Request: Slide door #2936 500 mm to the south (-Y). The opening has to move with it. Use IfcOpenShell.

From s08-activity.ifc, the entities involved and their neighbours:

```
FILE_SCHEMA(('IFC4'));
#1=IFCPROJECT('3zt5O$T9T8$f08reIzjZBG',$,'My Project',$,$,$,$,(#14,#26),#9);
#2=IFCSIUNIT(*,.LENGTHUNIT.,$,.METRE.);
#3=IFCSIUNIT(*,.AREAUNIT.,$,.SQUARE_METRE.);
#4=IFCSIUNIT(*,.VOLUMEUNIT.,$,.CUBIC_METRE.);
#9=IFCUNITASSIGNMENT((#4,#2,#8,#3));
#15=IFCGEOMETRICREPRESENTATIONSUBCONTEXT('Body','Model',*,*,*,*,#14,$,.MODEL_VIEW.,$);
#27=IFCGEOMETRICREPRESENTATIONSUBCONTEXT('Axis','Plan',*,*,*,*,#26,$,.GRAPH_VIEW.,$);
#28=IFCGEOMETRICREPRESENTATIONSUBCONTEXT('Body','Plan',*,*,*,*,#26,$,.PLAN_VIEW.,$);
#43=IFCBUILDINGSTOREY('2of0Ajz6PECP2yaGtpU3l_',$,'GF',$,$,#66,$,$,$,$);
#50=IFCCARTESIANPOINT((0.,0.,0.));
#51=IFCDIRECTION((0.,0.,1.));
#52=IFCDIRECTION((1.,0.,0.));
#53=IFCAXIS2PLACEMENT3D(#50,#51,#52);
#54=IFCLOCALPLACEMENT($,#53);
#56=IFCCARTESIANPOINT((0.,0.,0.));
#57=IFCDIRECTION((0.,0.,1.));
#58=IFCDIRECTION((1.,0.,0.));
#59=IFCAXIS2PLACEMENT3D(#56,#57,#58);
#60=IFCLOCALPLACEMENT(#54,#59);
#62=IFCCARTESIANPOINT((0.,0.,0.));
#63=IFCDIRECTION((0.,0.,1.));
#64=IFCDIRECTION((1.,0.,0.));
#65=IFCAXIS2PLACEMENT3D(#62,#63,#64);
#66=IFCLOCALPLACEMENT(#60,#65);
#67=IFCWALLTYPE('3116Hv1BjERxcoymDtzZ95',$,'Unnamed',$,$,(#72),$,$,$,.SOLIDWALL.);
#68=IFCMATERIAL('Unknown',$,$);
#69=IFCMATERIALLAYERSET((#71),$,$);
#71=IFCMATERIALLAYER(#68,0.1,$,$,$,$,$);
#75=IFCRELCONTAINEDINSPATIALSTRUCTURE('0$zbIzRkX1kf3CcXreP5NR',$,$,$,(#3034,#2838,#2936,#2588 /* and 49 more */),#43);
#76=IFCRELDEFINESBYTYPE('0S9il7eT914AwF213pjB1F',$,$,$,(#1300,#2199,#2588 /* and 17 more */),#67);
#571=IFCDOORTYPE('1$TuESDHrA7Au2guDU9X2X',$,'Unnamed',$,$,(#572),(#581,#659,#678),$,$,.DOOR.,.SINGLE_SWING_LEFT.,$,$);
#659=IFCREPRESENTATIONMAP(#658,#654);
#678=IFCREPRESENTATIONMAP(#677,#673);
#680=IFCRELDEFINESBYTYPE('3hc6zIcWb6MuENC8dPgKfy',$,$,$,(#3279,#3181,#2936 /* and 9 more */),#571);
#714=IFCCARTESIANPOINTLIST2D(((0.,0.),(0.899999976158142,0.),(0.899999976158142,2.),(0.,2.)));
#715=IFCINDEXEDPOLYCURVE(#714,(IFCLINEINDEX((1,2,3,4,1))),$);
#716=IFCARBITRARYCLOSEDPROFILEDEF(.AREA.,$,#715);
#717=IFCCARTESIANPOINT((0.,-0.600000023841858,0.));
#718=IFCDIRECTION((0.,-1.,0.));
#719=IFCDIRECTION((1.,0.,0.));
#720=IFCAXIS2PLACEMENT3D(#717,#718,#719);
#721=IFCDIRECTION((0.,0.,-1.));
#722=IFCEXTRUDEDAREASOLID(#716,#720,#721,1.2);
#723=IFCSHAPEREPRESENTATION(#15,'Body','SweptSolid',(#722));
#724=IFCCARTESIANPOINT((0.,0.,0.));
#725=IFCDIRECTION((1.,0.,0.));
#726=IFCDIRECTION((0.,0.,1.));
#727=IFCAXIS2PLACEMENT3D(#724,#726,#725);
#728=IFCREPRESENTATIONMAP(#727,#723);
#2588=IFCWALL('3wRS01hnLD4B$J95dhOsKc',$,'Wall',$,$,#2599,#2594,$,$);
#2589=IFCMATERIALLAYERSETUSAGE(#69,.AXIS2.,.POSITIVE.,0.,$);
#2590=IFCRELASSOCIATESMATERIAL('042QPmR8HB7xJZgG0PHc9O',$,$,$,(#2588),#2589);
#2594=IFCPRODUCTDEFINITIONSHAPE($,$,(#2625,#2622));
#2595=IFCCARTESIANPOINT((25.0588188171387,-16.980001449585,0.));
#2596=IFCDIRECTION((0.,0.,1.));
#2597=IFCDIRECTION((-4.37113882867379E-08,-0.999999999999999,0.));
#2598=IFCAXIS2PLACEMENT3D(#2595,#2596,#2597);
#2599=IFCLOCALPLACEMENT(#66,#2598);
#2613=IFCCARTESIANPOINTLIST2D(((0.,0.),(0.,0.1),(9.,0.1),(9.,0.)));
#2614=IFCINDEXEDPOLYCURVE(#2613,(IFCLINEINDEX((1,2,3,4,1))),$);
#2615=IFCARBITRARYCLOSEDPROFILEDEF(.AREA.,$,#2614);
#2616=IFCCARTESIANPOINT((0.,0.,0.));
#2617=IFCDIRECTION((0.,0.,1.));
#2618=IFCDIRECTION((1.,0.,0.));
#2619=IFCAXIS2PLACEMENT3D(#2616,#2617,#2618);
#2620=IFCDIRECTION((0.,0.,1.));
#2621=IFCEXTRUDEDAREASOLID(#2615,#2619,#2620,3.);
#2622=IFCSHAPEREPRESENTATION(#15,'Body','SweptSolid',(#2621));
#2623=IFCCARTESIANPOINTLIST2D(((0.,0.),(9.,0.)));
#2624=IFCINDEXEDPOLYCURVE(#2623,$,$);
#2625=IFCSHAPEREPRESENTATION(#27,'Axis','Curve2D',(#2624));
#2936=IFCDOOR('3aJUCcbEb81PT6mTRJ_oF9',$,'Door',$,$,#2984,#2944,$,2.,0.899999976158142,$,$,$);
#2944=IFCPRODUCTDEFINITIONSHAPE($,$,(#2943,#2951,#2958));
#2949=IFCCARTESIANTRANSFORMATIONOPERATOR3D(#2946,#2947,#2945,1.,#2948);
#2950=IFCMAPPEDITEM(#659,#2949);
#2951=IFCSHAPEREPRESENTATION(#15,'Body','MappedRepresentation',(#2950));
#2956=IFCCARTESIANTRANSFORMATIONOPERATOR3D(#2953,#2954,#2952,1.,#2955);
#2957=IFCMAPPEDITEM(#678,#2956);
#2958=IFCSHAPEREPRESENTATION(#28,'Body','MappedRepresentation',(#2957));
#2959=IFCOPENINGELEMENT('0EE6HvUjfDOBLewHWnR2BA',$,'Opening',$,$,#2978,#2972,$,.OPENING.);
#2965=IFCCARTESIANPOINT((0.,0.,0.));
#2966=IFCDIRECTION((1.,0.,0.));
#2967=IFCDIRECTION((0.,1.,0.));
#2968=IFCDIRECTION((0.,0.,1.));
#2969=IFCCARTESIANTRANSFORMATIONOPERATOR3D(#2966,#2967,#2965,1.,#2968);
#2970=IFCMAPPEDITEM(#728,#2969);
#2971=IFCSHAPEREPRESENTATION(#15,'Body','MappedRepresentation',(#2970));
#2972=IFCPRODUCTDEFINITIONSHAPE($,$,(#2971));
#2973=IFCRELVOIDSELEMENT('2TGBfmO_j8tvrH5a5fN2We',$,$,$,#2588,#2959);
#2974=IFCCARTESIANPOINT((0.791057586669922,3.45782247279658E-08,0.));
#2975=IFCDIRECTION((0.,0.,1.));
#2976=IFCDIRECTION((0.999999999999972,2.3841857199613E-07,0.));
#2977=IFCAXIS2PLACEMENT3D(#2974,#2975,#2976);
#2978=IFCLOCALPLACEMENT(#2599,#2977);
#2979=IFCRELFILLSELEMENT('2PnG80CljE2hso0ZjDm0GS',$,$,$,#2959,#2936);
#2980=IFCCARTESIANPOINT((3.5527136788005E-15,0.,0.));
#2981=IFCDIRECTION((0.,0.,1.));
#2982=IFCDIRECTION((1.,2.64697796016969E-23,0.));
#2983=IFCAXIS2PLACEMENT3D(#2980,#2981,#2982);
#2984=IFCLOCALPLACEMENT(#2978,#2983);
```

```python
import ifcopenshell
import ifcopenshell.api.geometry
import ifcopenshell.util.placement
import ifcopenshell.util.unit

model = ifcopenshell.open("s08-activity.ifc")
unit_scale = ifcopenshell.util.unit.calculate_unit_scale(model)

door = model.by_guid("3aJUCcbEb81PT6mTRJ_oF9")
opening = door.FillsVoids[0].RelatingOpeningElement
wall = opening.VoidsElements[0].RelatingBuildingElement

wall_matrix = ifcopenshell.util.placement.get_local_placement(wall.ObjectPlacement)
shift = wall_matrix[:3, 0] * 0.5 / unit_scale
before = ifcopenshell.util.placement.get_local_placement(door.ObjectPlacement)[:3, 3].copy()

# The door is placed relative to its opening, so it follows when the opening moves.
matrix = ifcopenshell.util.placement.get_local_placement(opening.ObjectPlacement)
matrix[:3, 3] += shift
ifcopenshell.api.geometry.edit_object_placement(
    model, product=opening, matrix=matrix, is_si=False, should_transform_children=True
)

after = ifcopenshell.util.placement.get_local_placement(door.ObjectPlacement)[:3, 3]
print("door moved by", (after - before).round(3) + 0.0)

model.write("s08-activity_updated.ifc")
```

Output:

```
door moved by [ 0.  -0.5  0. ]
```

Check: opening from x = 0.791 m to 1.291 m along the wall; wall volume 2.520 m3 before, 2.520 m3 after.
